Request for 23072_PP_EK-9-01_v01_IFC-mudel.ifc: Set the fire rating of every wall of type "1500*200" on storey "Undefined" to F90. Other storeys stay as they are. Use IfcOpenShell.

First a look at what the model holds.

```python
import ifcopenshell
import ifcopenshell.util.element

model = ifcopenshell.open("23072_PP_EK-9-01_v01_IFC-mudel.ifc")
print(model.schema)
storey = next(s for s in model.by_type("IfcBuildingStorey") if s.Name == "Undefined")
walls = [e for e in ifcopenshell.util.element.get_decomposition(storey) if e.is_a("IfcWall")]
seen = {}
for e in walls:
    element_type = ifcopenshell.util.element.get_type(e)
    key = (element_type.Name if element_type != e and element_type else None, ifcopenshell.util.element.get_pset(e, "Pset_WallCommon", "FireRating"))
    seen[key] = seen.get(key, 0) + 1
for (name, value), count in sorted(seen.items(), key=str):
    print(count, "x", name, "|", value)
```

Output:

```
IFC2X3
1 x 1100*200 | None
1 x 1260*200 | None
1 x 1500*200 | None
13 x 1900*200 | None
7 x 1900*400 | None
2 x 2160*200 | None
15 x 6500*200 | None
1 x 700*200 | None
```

```python
import ifcopenshell
import ifcopenshell.api.pset
import ifcopenshell.util.element

model = ifcopenshell.open("23072_PP_EK-9-01_v01_IFC-mudel.ifc")

storey = next(s for s in model.by_type("IfcBuildingStorey") if s.Name == "Undefined")
walls = [e for e in ifcopenshell.util.element.get_decomposition(storey) if e.is_a("IfcWall")]

count = 0
for e in walls:
    element_type = ifcopenshell.util.element.get_type(e)
    if element_type in (None, e) or element_type.Name != "1500*200":
        continue
    # add_pset returns the element's existing set when there is one.
    pset = ifcopenshell.api.pset.add_pset(model, product=e, name="Pset_WallCommon")
    ifcopenshell.api.pset.edit_pset(model, pset=pset, properties={"FireRating": "F90"})
    count += 1

print(count, "walls updated")

model.write("23072_PP_EK-9-01_v01_IFC-mudel_edited.ifc")
```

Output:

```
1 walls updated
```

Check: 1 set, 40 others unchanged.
